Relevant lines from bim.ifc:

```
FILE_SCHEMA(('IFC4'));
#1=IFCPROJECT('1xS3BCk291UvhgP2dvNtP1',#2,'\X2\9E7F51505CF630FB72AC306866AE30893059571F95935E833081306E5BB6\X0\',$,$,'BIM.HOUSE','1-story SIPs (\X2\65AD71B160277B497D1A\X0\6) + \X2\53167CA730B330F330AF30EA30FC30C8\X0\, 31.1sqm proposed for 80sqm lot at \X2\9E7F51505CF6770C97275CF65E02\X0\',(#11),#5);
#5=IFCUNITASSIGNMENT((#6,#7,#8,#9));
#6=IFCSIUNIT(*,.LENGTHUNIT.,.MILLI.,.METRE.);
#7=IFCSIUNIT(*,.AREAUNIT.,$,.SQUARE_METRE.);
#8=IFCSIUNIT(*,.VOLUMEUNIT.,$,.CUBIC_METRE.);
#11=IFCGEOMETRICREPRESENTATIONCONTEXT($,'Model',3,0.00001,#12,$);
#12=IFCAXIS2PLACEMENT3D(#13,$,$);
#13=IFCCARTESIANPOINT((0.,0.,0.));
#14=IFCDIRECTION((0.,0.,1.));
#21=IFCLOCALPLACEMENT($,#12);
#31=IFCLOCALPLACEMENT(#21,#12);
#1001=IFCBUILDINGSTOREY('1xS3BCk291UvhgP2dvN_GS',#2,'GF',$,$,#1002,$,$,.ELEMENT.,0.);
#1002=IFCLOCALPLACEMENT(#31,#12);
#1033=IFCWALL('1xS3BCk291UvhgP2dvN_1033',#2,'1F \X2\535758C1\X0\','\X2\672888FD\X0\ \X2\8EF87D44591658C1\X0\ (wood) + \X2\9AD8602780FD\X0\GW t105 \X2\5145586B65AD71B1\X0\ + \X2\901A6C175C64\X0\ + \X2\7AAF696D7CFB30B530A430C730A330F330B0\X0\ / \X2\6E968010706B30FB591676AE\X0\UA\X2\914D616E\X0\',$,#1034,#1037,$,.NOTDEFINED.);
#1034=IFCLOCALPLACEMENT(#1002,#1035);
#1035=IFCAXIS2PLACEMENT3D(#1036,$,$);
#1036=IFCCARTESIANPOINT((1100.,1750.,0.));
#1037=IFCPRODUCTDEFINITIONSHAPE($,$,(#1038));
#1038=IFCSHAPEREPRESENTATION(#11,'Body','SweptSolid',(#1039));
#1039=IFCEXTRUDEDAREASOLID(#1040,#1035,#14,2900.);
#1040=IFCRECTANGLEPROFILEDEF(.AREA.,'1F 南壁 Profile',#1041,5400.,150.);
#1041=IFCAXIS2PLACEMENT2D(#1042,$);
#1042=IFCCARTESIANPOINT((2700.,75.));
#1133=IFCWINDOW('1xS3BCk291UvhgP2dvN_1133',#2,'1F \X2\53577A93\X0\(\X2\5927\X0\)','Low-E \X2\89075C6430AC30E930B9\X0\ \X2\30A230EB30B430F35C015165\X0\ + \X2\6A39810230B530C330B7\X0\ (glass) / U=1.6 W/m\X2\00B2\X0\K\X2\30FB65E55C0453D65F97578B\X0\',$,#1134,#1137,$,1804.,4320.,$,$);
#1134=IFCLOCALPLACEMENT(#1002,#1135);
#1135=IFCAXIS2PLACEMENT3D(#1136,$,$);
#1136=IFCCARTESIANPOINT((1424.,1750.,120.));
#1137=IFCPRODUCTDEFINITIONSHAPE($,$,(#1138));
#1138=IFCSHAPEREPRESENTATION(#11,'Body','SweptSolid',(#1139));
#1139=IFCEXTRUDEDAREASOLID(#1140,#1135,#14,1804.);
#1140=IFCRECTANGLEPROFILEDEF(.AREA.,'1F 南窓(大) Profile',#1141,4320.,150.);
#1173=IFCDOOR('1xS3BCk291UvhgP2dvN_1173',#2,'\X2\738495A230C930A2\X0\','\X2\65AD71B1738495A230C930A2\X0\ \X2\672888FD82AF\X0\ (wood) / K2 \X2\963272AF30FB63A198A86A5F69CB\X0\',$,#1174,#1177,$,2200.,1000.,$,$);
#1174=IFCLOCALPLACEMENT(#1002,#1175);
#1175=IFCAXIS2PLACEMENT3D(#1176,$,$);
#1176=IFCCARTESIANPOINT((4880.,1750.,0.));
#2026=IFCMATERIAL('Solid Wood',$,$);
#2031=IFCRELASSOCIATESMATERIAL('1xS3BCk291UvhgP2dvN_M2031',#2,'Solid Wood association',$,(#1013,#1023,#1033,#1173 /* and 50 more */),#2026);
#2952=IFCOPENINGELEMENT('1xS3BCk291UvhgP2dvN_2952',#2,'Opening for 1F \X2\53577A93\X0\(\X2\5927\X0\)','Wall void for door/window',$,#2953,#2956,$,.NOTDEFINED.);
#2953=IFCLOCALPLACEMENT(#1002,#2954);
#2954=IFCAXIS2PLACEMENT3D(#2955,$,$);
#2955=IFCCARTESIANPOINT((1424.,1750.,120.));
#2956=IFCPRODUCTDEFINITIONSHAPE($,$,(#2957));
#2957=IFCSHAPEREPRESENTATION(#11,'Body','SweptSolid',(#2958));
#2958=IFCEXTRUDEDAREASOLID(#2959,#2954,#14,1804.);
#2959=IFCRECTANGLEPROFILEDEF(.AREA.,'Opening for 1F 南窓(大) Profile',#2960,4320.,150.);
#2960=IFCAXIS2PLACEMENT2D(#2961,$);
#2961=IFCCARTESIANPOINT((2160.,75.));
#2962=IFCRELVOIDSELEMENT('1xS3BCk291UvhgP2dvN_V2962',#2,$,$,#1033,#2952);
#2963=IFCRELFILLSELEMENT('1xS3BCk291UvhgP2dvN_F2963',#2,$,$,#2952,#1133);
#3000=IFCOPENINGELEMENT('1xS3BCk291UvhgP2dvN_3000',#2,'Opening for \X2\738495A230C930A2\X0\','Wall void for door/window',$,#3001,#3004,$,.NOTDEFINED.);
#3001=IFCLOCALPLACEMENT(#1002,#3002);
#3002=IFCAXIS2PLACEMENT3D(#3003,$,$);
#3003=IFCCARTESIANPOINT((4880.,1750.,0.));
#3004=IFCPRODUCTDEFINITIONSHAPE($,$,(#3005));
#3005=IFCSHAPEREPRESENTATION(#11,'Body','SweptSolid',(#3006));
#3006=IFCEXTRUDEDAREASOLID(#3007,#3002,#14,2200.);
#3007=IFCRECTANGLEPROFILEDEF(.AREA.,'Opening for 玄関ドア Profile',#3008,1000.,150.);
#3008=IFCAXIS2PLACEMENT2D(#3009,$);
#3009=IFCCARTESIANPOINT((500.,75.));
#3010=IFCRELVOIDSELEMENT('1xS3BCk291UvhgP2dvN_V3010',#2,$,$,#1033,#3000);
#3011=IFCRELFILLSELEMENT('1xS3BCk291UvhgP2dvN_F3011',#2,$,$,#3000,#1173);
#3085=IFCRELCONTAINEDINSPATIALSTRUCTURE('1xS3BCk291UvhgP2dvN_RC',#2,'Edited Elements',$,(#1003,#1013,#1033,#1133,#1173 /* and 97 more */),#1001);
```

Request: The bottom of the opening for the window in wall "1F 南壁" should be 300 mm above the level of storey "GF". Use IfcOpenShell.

```python
import numpy as np
import ifcopenshell
import ifcopenshell.api.geometry
import ifcopenshell.geom
import ifcopenshell.util.element
import ifcopenshell.util.placement
import ifcopenshell.util.shape
import ifcopenshell.util.unit

model = ifcopenshell.open("bim.ifc")
unit_scale = ifcopenshell.util.unit.calculate_unit_scale(model)

window = model.by_guid("1xS3BCk291UvhgP2dvN_1133")
opening = window.FillsVoids[0].RelatingOpeningElement
storey = ifcopenshell.util.element.get_container(window, ifc_class="IfcBuildingStorey")
level = ifcopenshell.util.placement.get_local_placement(storey.ObjectPlacement)[2, 3]

# The opening's origin need not be at the sill, so measure its lowest point.
shape = ifcopenshell.geom.create_shape(ifcopenshell.geom.settings(), opening)
bottom = ifcopenshell.util.shape.get_shape_bottom_elevation(shape, shape.geometry) / unit_scale
dz = level + 0.3 / unit_scale - bottom

shift = np.array([0.0, 0.0, dz])
# The window is not placed relative to its opening, so move both.
for product in (opening, window):
    matrix = ifcopenshell.util.placement.get_local_placement(product.ObjectPlacement)
    matrix[:3, 3] += shift
    ifcopenshell.api.geometry.edit_object_placement(model, product=product, matrix=matrix, is_si=False)

print(f"moved by {dz * unit_scale:+.3f} m")

model.write("bim_updated.ifc")
```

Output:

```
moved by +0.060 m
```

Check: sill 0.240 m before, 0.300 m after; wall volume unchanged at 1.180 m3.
